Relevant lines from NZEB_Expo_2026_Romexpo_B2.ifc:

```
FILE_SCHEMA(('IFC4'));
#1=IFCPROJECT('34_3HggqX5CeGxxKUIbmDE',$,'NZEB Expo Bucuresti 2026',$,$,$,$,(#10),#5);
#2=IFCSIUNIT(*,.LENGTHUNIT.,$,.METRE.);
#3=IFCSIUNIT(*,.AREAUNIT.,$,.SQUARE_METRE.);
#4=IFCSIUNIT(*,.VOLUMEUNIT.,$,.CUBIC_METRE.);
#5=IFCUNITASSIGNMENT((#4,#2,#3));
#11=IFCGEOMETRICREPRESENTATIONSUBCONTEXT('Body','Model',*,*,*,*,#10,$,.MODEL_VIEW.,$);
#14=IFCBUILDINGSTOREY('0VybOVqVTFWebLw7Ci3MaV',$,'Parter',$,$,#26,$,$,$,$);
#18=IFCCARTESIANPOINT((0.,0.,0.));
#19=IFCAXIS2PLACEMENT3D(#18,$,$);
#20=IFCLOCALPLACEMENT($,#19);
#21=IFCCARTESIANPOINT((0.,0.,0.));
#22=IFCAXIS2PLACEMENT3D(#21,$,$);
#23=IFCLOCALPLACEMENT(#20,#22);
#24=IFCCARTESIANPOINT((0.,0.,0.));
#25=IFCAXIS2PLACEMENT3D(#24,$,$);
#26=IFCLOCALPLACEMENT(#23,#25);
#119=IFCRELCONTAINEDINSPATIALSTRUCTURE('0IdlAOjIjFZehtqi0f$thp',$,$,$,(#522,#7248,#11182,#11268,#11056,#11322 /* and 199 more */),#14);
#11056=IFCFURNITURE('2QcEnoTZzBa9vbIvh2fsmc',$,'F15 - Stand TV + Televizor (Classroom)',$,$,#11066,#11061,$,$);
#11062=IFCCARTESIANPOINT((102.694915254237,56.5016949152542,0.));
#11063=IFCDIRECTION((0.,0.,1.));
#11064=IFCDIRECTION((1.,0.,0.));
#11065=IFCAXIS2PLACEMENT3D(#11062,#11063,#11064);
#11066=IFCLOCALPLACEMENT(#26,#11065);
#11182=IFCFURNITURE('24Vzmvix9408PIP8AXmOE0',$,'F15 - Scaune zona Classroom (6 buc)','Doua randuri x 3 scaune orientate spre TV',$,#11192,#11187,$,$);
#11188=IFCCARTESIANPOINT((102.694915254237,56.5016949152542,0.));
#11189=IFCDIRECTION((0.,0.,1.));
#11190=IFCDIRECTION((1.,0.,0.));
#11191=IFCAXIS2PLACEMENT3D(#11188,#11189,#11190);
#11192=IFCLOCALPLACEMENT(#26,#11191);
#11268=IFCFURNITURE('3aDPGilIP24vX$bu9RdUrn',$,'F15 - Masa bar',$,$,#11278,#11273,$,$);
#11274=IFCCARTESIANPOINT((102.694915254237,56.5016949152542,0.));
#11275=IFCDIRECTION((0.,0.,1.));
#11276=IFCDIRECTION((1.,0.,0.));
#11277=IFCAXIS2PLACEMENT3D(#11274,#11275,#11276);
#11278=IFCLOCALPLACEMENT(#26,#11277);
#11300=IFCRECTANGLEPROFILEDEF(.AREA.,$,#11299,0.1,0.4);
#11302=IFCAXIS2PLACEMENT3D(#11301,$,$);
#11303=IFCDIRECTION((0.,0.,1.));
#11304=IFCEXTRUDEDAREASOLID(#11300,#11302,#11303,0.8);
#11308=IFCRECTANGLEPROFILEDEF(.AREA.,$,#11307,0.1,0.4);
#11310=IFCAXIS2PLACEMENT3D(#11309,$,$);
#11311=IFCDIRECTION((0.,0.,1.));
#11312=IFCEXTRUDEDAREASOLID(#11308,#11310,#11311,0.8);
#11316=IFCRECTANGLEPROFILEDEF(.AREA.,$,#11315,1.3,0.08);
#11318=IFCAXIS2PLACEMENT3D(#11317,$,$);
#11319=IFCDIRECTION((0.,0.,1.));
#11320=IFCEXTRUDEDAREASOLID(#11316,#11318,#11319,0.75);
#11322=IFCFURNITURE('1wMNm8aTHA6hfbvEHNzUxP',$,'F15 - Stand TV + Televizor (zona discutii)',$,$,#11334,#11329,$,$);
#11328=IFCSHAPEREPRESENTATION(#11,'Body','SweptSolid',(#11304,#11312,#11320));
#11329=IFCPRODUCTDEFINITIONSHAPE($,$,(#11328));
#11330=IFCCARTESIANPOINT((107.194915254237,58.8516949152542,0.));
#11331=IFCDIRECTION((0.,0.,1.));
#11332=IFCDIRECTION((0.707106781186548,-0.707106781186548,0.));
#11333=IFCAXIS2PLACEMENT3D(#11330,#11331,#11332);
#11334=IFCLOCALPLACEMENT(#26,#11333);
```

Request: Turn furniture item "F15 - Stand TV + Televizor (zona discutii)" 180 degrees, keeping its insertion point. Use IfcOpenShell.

```python
import ifcopenshell
import ifcopenshell.api.geometry
import ifcopenshell.util.placement

model = ifcopenshell.open("NZEB_Expo_2026_Romexpo_B2.ifc")

item = model.by_guid("1wMNm8aTHA6hfbvEHNzUxP")
matrix = ifcopenshell.util.placement.get_local_placement(item.ObjectPlacement)
matrix = matrix @ ifcopenshell.util.placement.rotation(180, "Z")
ifcopenshell.api.geometry.edit_object_placement(model, product=item, matrix=matrix, is_si=False)

print(ifcopenshell.util.placement.get_local_placement(item.ObjectPlacement).round(3) + 0.0)

model.write("NZEB_Expo_2026_Romexpo_B2_edited.ifc")
```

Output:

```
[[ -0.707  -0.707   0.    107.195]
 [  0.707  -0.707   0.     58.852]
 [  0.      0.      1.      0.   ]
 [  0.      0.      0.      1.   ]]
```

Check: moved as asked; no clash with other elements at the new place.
